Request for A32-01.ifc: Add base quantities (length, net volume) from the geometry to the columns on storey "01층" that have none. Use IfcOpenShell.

First a look at what the model holds.

```python
import ifcopenshell
import ifcopenshell.util.element
import ifcopenshell.util.unit

model = ifcopenshell.open("A32-01.ifc")
print(model.schema)
for unit_type in ("LENGTHUNIT", "AREAUNIT", "VOLUMEUNIT"):
    print(unit_type, ifcopenshell.util.unit.calculate_unit_scale(model, unit_type))
storey = next(s for s in model.by_type("IfcBuildingStorey") if s.Name == "01층")
columns = [e for e in ifcopenshell.util.element.get_decomposition(storey) if e.is_a("IfcColumn")]
for e in sorted(columns, key=lambda e: e.id()):
    print(e.id(), e.is_a(), e.Name, list(ifcopenshell.util.element.get_psets(e, qtos_only=True)), sep=" | ")
```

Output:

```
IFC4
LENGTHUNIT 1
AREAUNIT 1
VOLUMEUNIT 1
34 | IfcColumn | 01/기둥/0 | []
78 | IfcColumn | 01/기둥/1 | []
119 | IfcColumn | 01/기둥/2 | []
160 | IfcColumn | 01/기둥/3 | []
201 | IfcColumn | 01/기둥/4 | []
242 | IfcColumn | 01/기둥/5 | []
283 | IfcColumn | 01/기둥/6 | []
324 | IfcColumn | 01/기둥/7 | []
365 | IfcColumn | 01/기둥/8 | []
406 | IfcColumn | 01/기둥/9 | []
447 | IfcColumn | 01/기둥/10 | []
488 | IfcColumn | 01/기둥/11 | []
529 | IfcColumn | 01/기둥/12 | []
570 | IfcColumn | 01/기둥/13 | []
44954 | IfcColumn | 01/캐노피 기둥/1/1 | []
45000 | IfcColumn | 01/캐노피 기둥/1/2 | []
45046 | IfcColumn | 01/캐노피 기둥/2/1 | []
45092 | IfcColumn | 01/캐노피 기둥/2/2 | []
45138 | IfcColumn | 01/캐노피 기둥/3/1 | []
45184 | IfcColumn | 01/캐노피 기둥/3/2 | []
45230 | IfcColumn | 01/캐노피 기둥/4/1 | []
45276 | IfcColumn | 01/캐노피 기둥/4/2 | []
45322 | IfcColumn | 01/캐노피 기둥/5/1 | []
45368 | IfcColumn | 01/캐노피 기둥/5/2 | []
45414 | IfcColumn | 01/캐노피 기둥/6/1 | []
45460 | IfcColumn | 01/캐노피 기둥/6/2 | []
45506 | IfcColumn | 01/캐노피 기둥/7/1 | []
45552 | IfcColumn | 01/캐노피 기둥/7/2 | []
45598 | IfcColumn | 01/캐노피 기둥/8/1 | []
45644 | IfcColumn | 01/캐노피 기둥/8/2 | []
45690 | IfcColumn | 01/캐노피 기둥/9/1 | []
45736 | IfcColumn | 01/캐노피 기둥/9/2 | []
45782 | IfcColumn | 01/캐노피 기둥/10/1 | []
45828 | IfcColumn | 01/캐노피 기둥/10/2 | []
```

```python
import ifcopenshell
import ifcopenshell.api.pset
import ifcopenshell.geom
import ifcopenshell.util.element
import ifcopenshell.util.shape
import ifcopenshell.util.unit

model = ifcopenshell.open("A32-01.ifc")
unit_scale = ifcopenshell.util.unit.calculate_unit_scale(model)
volume_scale = ifcopenshell.util.unit.calculate_unit_scale(model, "VOLUMEUNIT")
settings = ifcopenshell.geom.settings()

storey = next(s for s in model.by_type("IfcBuildingStorey") if s.Name == "01층")
columns = [e for e in ifcopenshell.util.element.get_decomposition(storey) if e.is_a("IfcColumn")]

for e in sorted(columns, key=lambda e: e.id()):
    if ifcopenshell.util.element.get_psets(e, qtos_only=True, should_inherit=False):
        continue
    # Geometry comes back in metres, in the element's own axes.
    shape = ifcopenshell.geom.create_shape(settings, e)
    values = {
        "Length": ifcopenshell.util.shape.get_z(shape.geometry) / unit_scale,
        "NetVolume": ifcopenshell.util.shape.get_volume(shape.geometry) / volume_scale,
    }
    qto = ifcopenshell.api.pset.add_qto(model, product=e, name="Qto_ColumnBaseQuantities")
    ifcopenshell.api.pset.edit_qto(model, qto=qto, properties=values)
    print(e.id(), {k: round(v, 3) for k, v in values.items()})

model.write("A32-01_updated.ifc")
```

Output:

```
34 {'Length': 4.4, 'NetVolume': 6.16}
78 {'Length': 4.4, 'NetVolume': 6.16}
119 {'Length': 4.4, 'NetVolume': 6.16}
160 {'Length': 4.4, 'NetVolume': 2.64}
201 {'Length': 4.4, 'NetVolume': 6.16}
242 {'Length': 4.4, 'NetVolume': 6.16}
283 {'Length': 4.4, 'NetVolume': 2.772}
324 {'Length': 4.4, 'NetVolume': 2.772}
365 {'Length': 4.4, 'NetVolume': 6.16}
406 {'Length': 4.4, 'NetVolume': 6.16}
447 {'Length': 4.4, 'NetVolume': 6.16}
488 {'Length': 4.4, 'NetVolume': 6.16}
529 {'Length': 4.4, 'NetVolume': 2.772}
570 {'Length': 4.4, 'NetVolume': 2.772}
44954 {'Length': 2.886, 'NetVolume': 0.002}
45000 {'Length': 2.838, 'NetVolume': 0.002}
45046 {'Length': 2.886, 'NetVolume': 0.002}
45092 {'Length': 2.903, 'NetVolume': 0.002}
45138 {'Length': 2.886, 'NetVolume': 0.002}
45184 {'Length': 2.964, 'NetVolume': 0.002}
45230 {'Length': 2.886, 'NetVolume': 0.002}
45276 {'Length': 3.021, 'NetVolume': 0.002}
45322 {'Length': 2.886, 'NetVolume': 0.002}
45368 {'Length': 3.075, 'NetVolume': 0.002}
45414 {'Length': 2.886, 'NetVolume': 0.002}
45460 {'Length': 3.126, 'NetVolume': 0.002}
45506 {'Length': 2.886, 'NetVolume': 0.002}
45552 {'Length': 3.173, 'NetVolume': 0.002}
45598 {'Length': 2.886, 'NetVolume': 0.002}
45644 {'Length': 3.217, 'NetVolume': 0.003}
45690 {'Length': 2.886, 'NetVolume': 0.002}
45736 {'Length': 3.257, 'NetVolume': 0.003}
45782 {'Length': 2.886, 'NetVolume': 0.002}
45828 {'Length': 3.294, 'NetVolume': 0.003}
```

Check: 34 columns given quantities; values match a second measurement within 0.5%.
